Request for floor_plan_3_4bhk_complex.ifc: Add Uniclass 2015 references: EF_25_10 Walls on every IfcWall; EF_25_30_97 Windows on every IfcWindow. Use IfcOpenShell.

First a look at what the model holds.

```python
import ifcopenshell

model = ifcopenshell.open("floor_plan_3_4bhk_complex.ifc")
print(model.schema)
print("classifications:", [c.Name for c in model.by_type("IfcClassification")])
for ifc_class in ("IfcDoor", "IfcRoof", "IfcStair", "IfcWall", "IfcWindow"):
    print(ifc_class, len(model.by_type(ifc_class)))
```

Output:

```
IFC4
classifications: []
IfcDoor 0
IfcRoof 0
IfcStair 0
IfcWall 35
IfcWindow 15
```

```python
import ifcopenshell
import ifcopenshell.api.classification

model = ifcopenshell.open("floor_plan_3_4bhk_complex.ifc")

system = ifcopenshell.api.classification.add_classification(model, classification="Uniclass 2015")

codes = {
    "IfcWall": ("EF_25_10", "Walls"),
    "IfcWindow": ("EF_25_30_97", "Windows"),
}
for ifc_class, (code, name) in codes.items():
    products = model.by_type(ifc_class)
    ifcopenshell.api.classification.add_reference(
        model, products=products, classification=system, identification=code, name=name
    )
    print(code, len(products))

model.write("floor_plan_3_4bhk_complex_updated.ifc")
```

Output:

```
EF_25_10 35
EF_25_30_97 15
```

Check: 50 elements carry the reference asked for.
